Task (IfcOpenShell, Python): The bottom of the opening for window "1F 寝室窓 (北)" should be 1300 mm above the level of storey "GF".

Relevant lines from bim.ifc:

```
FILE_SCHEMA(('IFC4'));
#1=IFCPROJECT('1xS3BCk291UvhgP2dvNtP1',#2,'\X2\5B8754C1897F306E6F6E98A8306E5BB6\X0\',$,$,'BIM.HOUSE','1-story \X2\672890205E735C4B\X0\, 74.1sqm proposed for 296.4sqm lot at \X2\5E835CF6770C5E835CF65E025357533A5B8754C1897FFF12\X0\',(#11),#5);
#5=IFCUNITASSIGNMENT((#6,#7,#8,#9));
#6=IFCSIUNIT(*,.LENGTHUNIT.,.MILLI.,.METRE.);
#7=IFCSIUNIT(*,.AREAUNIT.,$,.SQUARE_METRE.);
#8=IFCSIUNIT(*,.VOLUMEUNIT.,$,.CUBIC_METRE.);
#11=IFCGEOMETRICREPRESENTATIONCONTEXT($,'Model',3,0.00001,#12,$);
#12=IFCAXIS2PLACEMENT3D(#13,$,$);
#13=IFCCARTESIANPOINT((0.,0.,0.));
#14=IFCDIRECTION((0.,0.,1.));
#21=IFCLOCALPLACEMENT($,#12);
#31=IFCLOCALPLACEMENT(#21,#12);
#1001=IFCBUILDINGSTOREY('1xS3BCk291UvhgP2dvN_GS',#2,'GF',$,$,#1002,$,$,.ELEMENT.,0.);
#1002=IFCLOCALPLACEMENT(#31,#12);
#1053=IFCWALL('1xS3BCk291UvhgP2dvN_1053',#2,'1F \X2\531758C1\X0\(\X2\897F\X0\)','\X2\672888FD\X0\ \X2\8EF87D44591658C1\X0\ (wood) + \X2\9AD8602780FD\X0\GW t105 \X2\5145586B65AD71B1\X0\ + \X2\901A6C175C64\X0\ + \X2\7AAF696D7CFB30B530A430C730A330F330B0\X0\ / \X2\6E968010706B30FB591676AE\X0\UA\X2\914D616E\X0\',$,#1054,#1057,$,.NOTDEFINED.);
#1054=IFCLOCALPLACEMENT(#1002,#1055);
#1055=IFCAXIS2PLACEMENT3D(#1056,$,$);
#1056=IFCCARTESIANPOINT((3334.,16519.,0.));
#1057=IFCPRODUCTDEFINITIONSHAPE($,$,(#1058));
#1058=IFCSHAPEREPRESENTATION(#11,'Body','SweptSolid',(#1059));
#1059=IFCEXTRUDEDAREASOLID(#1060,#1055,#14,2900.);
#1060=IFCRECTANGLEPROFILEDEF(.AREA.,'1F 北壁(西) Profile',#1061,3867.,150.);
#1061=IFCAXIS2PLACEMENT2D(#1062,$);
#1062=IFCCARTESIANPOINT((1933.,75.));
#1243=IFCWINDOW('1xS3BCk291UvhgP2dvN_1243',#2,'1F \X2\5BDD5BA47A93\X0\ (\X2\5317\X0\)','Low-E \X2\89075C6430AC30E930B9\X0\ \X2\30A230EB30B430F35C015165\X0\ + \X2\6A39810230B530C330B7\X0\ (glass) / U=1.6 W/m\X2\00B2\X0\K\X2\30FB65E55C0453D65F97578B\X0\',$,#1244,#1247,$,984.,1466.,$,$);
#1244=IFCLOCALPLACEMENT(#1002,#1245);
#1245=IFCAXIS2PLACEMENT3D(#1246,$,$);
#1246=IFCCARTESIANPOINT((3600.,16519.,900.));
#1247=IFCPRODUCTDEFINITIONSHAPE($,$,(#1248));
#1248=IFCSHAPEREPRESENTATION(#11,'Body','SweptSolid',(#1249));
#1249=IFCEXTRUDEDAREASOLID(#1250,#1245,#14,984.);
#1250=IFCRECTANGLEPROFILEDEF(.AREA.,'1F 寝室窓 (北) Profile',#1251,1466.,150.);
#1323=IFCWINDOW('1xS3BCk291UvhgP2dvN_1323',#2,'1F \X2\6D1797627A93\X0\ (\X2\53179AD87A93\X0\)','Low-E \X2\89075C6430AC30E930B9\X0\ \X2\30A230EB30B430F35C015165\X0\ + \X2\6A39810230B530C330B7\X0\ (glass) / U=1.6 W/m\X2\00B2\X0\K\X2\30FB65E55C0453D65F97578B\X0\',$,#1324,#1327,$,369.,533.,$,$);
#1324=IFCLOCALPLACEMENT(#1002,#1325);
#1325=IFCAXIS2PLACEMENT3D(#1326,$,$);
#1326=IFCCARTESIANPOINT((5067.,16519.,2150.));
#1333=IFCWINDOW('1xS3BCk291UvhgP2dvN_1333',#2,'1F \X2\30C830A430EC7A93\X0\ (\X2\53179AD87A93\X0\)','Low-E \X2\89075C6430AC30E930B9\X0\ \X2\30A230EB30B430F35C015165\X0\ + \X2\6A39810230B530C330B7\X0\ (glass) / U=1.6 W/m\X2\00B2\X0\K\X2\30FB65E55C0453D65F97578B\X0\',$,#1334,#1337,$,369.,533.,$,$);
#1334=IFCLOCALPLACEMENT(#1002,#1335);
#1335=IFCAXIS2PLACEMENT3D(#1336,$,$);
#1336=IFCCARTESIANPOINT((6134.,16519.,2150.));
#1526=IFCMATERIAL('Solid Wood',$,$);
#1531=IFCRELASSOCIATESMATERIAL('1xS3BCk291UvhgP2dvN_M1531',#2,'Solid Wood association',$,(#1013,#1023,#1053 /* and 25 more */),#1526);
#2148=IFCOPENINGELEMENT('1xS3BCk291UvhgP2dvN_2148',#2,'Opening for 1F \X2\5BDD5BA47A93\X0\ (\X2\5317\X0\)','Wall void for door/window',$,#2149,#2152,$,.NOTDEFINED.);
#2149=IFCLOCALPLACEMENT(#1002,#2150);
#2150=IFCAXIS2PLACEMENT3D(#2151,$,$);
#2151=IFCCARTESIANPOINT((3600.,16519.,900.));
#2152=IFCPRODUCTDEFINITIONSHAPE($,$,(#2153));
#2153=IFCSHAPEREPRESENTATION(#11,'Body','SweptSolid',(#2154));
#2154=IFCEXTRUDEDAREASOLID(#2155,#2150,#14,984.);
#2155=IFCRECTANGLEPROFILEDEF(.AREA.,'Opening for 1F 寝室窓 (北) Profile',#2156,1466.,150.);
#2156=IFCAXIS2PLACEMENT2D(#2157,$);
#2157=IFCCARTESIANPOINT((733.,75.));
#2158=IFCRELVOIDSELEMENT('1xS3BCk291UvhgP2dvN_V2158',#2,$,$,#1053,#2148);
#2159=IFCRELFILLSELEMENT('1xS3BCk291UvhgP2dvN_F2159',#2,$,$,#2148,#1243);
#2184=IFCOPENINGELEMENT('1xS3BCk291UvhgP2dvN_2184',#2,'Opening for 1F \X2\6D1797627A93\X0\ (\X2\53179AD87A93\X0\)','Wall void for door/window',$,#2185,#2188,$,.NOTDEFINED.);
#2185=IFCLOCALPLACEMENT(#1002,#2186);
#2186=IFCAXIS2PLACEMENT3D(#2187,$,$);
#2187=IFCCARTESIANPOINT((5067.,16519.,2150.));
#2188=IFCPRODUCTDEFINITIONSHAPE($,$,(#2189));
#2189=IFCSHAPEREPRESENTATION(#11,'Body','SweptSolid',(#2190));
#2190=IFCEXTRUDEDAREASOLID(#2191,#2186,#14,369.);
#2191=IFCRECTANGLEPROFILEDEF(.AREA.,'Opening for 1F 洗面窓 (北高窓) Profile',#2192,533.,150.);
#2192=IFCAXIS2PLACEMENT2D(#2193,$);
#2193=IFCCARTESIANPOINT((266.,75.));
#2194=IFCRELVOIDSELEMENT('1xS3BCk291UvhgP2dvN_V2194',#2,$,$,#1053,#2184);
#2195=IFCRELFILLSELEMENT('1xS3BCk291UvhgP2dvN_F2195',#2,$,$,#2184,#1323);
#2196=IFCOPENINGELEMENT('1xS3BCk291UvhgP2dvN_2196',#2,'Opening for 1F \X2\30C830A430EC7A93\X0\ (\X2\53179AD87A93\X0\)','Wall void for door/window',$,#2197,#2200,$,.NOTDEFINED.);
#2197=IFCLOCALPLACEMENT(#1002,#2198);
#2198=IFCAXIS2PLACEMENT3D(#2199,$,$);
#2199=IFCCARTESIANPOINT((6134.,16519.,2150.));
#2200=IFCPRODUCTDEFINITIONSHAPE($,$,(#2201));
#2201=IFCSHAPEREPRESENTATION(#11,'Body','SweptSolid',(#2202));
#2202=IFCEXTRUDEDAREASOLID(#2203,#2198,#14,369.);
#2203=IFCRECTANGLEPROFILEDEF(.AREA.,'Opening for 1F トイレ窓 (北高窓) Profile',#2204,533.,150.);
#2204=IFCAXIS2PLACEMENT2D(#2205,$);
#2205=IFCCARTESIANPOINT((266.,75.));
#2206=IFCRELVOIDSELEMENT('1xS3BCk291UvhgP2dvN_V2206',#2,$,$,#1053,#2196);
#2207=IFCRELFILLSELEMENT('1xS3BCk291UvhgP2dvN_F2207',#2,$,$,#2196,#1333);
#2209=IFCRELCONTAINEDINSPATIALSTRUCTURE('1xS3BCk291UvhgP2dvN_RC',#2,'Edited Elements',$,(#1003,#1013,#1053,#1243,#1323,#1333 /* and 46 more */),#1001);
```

```python
import numpy as np
import ifcopenshell
import ifcopenshell.api.geometry
import ifcopenshell.geom
import ifcopenshell.util.element
import ifcopenshell.util.placement
import ifcopenshell.util.shape
import ifcopenshell.util.unit

model = ifcopenshell.open("bim.ifc")
unit_scale = ifcopenshell.util.unit.calculate_unit_scale(model)

window = model.by_id(1243)
opening = window.FillsVoids[0].RelatingOpeningElement
storey = ifcopenshell.util.element.get_container(window, ifc_class="IfcBuildingStorey")
level = ifcopenshell.util.placement.get_local_placement(storey.ObjectPlacement)[2, 3]

# The opening's origin need not be at the sill, so measure its lowest point.
shape = ifcopenshell.geom.create_shape(ifcopenshell.geom.settings(), opening)
bottom = ifcopenshell.util.shape.get_shape_bottom_elevation(shape, shape.geometry) / unit_scale
dz = level + 1300.0 - bottom

shift = np.array([0.0, 0.0, dz])
# The window is not placed relative to its opening, so move both.
for product in (opening, window):
    matrix = ifcopenshell.util.placement.get_local_placement(product.ObjectPlacement)
    matrix[:3, 3] += shift
    ifcopenshell.api.geometry.edit_object_placement(model, product=product, matrix=matrix, is_si=False)

print(f"moved by {dz * unit_scale:+.3f} m")

model.write("bim_updated.ifc")
```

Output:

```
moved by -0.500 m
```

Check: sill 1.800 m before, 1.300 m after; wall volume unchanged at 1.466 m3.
